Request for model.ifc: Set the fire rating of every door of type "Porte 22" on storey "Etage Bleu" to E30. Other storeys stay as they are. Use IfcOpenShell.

First a look at what the model holds.

```python
import ifcopenshell
import ifcopenshell.util.element

model = ifcopenshell.open("model.ifc")
print(model.schema)
storey = next(s for s in model.by_type("IfcBuildingStorey") if s.Name == "Etage Bleu")
doors = [e for e in ifcopenshell.util.element.get_decomposition(storey) if e.is_a("IfcDoor")]
seen = {}
for e in doors:
    element_type = ifcopenshell.util.element.get_type(e)
    key = (element_type.Name if element_type != e and element_type else None, ifcopenshell.util.element.get_pset(e, "Pset_DoorCommon", "FireRating"))
    seen[key] = seen.get(key, 0) + 1
for (name, value), count in sorted(seen.items(), key=str):
    print(count, "x", name, "|", value)
```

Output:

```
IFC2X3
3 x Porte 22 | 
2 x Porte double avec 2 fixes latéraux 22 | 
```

```python
import ifcopenshell
import ifcopenshell.api.pset
import ifcopenshell.util.element

model = ifcopenshell.open("model.ifc")

storey = next(s for s in model.by_type("IfcBuildingStorey") if s.Name == "Etage Bleu")
doors = [e for e in ifcopenshell.util.element.get_decomposition(storey) if e.is_a("IfcDoor")]

count = 0
for e in doors:
    element_type = ifcopenshell.util.element.get_type(e)
    if element_type in (None, e) or element_type.Name != "Porte 22":
        continue
    # add_pset returns the element's existing set when there is one.
    pset = ifcopenshell.api.pset.add_pset(model, product=e, name="Pset_DoorCommon")
    ifcopenshell.api.pset.edit_pset(model, pset=pset, properties={"FireRating": "E30"})
    count += 1

print(count, "doors updated")

model.write("model_edited.ifc")
```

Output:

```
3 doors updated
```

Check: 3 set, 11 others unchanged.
